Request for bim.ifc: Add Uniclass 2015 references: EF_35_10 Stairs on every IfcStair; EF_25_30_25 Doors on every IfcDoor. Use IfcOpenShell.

First a look at what the model holds.

```python
import ifcopenshell

model = ifcopenshell.open("bim.ifc")
print(model.schema)
print("classifications:", [c.Name for c in model.by_type("IfcClassification")])
for ifc_class in ("IfcDoor", "IfcRoof", "IfcStair", "IfcWall", "IfcWindow"):
    print(ifc_class, len(model.by_type(ifc_class)))
```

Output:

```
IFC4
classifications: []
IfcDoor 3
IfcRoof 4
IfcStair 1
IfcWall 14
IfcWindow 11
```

```python
import ifcopenshell
import ifcopenshell.api.classification

model = ifcopenshell.open("bim.ifc")

system = ifcopenshell.api.classification.add_classification(model, classification="Uniclass 2015")

codes = {
    "IfcStair": ("EF_35_10", "Stairs"),
    "IfcDoor": ("EF_25_30_25", "Doors"),
}
for ifc_class, (code, name) in codes.items():
    products = model.by_type(ifc_class)
    ifcopenshell.api.classification.add_reference(
        model, products=products, classification=system, identification=code, name=name
    )
    print(code, len(products))

model.write("bim_rev.ifc")
```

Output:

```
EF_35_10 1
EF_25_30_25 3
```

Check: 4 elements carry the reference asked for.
